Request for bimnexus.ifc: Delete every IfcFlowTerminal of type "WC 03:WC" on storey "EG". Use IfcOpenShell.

First a look at what the model holds.

```python
import ifcopenshell
import ifcopenshell.util.element

model = ifcopenshell.open("bimnexus.ifc")
print(model.schema)
storey = next(s for s in model.by_type("IfcBuildingStorey") if s.Name == "EG")
terminals = [e for e in ifcopenshell.util.element.get_decomposition(storey) if e.is_a("IfcFlowTerminal")]
seen = {}
for e in terminals:
    element_type = ifcopenshell.util.element.get_type(e)
    name = element_type.Name if element_type not in (None, e) else None
    seen[name] = seen.get(name, 0) + 1
for name, count in sorted(seen.items(), key=str):
    print(count, "x", name)
```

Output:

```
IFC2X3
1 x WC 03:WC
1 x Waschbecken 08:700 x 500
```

```python
import ifcopenshell
import ifcopenshell.api.root
import ifcopenshell.util.element

model = ifcopenshell.open("bimnexus.ifc")

storey = next(s for s in model.by_type("IfcBuildingStorey") if s.Name == "EG")
terminals = [e for e in ifcopenshell.util.element.get_decomposition(storey) if e.is_a("IfcFlowTerminal")]
targets = [e for e in terminals if (t := ifcopenshell.util.element.get_type(e)) not in (None, e) and t.Name == "WC 03:WC"]

for e in targets:
    ifcopenshell.api.root.remove_product(model, product=e)
print(len(targets), "removed")

model.write("bimnexus_rev.ifc")
```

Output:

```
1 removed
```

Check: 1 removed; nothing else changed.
